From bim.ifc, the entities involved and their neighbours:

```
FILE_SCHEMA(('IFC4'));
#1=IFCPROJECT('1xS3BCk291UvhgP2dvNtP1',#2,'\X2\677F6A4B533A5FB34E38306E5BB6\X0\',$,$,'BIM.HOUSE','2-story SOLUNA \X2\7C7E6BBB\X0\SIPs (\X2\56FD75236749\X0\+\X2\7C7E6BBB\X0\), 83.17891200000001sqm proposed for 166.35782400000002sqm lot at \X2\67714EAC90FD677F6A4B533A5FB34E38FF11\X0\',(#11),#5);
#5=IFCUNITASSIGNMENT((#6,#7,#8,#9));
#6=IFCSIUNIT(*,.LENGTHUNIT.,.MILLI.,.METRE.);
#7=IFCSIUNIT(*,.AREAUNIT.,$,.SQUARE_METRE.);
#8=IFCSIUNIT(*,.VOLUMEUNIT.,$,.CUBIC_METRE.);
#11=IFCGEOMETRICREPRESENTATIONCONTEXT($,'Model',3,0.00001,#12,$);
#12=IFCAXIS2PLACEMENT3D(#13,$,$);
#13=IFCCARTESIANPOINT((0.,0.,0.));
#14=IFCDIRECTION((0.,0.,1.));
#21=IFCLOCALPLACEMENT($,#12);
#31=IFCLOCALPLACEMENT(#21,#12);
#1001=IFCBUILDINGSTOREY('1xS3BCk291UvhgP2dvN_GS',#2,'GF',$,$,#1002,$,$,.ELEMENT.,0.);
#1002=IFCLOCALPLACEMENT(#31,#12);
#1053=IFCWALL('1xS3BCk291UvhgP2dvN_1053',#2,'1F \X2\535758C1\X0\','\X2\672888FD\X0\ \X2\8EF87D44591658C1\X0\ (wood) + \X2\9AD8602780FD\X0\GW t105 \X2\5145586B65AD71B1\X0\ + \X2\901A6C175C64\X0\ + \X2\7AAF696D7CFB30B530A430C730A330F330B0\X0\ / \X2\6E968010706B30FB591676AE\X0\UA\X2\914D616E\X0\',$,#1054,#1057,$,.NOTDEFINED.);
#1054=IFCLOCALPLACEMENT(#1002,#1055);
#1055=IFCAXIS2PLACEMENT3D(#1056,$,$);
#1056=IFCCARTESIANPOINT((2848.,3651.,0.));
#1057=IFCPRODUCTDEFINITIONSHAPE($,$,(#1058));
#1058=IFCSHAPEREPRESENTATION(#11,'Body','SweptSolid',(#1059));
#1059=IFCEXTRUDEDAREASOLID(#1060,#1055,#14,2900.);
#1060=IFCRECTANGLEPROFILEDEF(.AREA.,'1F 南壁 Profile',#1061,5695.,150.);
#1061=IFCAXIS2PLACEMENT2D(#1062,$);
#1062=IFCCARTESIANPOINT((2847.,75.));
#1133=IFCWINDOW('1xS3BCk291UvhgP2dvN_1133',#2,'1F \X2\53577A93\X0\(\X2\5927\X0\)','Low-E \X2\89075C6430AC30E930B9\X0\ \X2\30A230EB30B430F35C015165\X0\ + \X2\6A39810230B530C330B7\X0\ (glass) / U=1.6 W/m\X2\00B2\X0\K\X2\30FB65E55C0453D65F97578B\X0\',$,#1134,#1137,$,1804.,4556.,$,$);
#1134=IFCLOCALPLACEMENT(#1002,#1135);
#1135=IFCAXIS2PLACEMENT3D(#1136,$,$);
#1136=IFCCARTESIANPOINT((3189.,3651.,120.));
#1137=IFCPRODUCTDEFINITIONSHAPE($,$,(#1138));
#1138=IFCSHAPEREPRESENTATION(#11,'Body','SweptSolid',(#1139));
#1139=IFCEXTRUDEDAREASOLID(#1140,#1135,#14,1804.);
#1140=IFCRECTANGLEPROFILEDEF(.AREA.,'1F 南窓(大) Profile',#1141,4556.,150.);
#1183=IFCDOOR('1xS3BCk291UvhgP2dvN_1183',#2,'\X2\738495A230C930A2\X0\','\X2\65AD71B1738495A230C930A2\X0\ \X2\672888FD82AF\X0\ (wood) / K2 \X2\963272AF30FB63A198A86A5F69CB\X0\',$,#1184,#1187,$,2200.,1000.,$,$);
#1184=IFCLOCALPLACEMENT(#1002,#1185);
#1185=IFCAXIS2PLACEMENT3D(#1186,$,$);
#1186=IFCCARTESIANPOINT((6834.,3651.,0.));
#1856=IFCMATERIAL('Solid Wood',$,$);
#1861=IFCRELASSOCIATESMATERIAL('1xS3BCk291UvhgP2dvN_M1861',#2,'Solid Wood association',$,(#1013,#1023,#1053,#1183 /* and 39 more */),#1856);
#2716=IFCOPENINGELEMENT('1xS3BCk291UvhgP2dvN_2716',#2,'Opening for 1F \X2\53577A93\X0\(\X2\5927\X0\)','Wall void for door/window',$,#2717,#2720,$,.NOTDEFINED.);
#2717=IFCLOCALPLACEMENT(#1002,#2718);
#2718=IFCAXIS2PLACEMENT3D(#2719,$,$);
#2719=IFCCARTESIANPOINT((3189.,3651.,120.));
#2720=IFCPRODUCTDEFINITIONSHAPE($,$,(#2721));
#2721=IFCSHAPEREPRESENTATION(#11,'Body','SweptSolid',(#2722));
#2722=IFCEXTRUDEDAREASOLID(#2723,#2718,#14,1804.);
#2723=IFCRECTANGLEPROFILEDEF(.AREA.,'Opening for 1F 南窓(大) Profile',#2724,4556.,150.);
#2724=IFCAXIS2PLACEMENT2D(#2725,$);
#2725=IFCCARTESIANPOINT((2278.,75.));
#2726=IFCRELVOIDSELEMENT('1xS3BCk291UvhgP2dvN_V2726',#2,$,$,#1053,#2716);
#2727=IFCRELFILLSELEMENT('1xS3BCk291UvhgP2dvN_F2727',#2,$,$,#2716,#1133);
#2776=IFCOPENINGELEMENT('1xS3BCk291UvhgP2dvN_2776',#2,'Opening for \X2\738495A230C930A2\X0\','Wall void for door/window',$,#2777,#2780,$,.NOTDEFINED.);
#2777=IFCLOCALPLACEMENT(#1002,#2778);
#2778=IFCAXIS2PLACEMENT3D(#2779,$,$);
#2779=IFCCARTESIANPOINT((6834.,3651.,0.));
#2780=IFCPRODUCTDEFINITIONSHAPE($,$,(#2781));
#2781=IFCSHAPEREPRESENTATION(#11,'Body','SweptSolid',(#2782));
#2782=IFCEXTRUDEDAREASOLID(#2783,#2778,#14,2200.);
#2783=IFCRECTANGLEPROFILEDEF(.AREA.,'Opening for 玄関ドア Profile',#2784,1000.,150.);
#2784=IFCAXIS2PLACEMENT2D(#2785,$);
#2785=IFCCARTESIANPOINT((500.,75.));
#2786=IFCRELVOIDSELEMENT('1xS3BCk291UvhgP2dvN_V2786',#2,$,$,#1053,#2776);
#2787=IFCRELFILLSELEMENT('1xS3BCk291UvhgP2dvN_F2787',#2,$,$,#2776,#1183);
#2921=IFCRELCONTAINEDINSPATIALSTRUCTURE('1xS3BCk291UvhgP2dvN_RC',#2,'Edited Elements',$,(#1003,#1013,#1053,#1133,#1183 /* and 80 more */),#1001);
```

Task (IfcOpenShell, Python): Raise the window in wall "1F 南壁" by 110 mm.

```python
import numpy as np
import ifcopenshell
import ifcopenshell.api.geometry
import ifcopenshell.util.placement
import ifcopenshell.util.unit

model = ifcopenshell.open("bim.ifc")
unit_scale = ifcopenshell.util.unit.calculate_unit_scale(model)

window = model.by_guid("1xS3BCk291UvhgP2dvN_1133")
opening = window.FillsVoids[0].RelatingOpeningElement
dz = 0.11 / unit_scale

shift = np.array([0.0, 0.0, dz])
# The window is not placed relative to its opening, so move both.
for product in (opening, window):
    matrix = ifcopenshell.util.placement.get_local_placement(product.ObjectPlacement)
    matrix[:3, 3] += shift
    ifcopenshell.api.geometry.edit_object_placement(model, product=product, matrix=matrix, is_si=False)

print(f"moved by {dz * unit_scale:+.3f} m")

model.write("bim_edited.ifc")
```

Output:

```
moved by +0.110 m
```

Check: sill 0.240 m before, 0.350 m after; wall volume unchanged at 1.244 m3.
